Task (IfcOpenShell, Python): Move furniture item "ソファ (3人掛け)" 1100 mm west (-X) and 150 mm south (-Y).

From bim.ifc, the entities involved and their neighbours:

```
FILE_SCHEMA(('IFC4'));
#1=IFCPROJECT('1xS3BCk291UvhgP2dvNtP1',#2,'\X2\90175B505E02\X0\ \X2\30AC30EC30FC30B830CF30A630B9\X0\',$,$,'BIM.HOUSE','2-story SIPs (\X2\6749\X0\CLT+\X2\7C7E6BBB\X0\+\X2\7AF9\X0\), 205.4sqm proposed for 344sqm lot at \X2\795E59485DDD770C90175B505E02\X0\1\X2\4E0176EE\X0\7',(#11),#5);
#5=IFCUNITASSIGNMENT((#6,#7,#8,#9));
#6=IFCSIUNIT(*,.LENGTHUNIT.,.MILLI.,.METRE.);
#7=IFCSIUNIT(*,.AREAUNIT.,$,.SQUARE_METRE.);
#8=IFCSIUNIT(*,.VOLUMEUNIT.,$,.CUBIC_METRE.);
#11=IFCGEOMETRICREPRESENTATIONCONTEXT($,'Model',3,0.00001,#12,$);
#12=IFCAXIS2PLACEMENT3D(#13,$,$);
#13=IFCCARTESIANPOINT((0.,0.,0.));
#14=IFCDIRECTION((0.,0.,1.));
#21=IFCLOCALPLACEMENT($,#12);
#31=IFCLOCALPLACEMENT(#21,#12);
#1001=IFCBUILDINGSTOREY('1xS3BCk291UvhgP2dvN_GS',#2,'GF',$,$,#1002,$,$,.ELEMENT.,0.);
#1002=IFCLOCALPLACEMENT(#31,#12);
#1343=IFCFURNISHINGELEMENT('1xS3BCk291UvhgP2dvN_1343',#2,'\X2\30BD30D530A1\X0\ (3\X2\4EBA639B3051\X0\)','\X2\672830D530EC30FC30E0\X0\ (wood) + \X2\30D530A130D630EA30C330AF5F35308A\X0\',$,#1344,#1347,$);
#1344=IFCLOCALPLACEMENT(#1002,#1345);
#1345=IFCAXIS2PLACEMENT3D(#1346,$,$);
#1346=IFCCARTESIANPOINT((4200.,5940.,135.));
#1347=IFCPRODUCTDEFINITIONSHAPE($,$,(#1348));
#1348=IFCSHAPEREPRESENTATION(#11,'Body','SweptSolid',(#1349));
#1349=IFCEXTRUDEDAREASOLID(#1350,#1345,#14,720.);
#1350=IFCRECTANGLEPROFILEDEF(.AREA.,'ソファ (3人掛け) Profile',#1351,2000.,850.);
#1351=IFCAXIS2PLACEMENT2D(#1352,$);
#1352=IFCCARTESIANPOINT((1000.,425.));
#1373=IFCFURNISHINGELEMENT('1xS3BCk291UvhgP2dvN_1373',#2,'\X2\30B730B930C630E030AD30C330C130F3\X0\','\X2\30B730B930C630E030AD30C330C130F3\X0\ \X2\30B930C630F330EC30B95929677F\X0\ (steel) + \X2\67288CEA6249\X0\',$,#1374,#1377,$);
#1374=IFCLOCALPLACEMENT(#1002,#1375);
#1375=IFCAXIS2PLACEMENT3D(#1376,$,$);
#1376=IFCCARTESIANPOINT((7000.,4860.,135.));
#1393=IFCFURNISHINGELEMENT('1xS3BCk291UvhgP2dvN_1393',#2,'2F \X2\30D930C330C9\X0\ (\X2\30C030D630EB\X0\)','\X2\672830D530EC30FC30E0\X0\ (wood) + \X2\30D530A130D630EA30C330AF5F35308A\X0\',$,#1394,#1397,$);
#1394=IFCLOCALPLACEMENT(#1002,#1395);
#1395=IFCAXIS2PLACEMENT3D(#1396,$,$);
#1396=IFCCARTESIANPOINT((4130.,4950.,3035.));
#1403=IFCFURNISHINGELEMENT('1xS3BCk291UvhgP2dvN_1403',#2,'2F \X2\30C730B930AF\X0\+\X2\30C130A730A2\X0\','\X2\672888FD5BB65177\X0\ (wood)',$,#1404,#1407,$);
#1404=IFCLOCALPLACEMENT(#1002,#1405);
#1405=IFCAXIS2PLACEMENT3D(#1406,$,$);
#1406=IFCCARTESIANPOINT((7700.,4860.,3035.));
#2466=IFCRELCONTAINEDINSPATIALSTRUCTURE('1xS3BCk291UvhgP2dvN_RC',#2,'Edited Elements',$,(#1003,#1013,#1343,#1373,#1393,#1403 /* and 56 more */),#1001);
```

```python
import ifcopenshell
import ifcopenshell.api.geometry
import ifcopenshell.util.placement
import ifcopenshell.util.unit

model = ifcopenshell.open("bim.ifc")
unit_scale = ifcopenshell.util.unit.calculate_unit_scale(model)

item = model.by_guid("1xS3BCk291UvhgP2dvN_1343")
matrix = ifcopenshell.util.placement.get_local_placement(item.ObjectPlacement)
matrix[0, 3] -= 1.1 / unit_scale
matrix[1, 3] -= 0.15 / unit_scale
ifcopenshell.api.geometry.edit_object_placement(model, product=item, matrix=matrix, is_si=False)

print(ifcopenshell.util.placement.get_local_placement(item.ObjectPlacement).round(3) + 0.0)

model.write("bim-out.ifc")
```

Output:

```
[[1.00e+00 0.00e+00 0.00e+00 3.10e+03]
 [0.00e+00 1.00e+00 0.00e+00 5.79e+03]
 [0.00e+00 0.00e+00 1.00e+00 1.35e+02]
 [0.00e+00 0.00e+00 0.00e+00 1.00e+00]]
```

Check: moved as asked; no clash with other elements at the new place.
